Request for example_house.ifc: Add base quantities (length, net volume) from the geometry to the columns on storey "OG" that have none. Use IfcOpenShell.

First a look at what the model holds.

```python
import ifcopenshell
import ifcopenshell.util.element
import ifcopenshell.util.unit

model = ifcopenshell.open("example_house.ifc")
print(model.schema)
for unit_type in ("LENGTHUNIT", "AREAUNIT", "VOLUMEUNIT"):
    print(unit_type, ifcopenshell.util.unit.calculate_unit_scale(model, unit_type))
storey = next(s for s in model.by_type("IfcBuildingStorey") if s.Name == "OG")
columns = [e for e in ifcopenshell.util.element.get_decomposition(storey) if e.is_a("IfcColumn")]
for e in sorted(columns, key=lambda e: e.id()):
    print(e.id(), e.is_a(), e.Name, list(ifcopenshell.util.element.get_psets(e, qtos_only=True)), sep=" | ")
```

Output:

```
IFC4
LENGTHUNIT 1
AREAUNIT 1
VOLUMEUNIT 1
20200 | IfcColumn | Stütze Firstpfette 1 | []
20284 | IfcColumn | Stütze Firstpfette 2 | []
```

```python
import ifcopenshell
import ifcopenshell.api.pset
import ifcopenshell.geom
import ifcopenshell.util.element
import ifcopenshell.util.shape
import ifcopenshell.util.unit

model = ifcopenshell.open("example_house.ifc")
unit_scale = ifcopenshell.util.unit.calculate_unit_scale(model)
volume_scale = ifcopenshell.util.unit.calculate_unit_scale(model, "VOLUMEUNIT")
settings = ifcopenshell.geom.settings()

storey = next(s for s in model.by_type("IfcBuildingStorey") if s.Name == "OG")
columns = [e for e in ifcopenshell.util.element.get_decomposition(storey) if e.is_a("IfcColumn")]

for e in sorted(columns, key=lambda e: e.id()):
    if ifcopenshell.util.element.get_psets(e, qtos_only=True, should_inherit=False):
        continue
    # Geometry comes back in metres, in the element's own axes.
    shape = ifcopenshell.geom.create_shape(settings, e)
    values = {
        "Length": ifcopenshell.util.shape.get_z(shape.geometry) / unit_scale,
        "NetVolume": ifcopenshell.util.shape.get_volume(shape.geometry) / volume_scale,
    }
    qto = ifcopenshell.api.pset.add_qto(model, product=e, name="Qto_ColumnBaseQuantities")
    ifcopenshell.api.pset.edit_qto(model, qto=qto, properties=values)
    print(e.id(), {k: round(v, 3) for k, v in values.items()})

model.write("example_house-out.ifc")
```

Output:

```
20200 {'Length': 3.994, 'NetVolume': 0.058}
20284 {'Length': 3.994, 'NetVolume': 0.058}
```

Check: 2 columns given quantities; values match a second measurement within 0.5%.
